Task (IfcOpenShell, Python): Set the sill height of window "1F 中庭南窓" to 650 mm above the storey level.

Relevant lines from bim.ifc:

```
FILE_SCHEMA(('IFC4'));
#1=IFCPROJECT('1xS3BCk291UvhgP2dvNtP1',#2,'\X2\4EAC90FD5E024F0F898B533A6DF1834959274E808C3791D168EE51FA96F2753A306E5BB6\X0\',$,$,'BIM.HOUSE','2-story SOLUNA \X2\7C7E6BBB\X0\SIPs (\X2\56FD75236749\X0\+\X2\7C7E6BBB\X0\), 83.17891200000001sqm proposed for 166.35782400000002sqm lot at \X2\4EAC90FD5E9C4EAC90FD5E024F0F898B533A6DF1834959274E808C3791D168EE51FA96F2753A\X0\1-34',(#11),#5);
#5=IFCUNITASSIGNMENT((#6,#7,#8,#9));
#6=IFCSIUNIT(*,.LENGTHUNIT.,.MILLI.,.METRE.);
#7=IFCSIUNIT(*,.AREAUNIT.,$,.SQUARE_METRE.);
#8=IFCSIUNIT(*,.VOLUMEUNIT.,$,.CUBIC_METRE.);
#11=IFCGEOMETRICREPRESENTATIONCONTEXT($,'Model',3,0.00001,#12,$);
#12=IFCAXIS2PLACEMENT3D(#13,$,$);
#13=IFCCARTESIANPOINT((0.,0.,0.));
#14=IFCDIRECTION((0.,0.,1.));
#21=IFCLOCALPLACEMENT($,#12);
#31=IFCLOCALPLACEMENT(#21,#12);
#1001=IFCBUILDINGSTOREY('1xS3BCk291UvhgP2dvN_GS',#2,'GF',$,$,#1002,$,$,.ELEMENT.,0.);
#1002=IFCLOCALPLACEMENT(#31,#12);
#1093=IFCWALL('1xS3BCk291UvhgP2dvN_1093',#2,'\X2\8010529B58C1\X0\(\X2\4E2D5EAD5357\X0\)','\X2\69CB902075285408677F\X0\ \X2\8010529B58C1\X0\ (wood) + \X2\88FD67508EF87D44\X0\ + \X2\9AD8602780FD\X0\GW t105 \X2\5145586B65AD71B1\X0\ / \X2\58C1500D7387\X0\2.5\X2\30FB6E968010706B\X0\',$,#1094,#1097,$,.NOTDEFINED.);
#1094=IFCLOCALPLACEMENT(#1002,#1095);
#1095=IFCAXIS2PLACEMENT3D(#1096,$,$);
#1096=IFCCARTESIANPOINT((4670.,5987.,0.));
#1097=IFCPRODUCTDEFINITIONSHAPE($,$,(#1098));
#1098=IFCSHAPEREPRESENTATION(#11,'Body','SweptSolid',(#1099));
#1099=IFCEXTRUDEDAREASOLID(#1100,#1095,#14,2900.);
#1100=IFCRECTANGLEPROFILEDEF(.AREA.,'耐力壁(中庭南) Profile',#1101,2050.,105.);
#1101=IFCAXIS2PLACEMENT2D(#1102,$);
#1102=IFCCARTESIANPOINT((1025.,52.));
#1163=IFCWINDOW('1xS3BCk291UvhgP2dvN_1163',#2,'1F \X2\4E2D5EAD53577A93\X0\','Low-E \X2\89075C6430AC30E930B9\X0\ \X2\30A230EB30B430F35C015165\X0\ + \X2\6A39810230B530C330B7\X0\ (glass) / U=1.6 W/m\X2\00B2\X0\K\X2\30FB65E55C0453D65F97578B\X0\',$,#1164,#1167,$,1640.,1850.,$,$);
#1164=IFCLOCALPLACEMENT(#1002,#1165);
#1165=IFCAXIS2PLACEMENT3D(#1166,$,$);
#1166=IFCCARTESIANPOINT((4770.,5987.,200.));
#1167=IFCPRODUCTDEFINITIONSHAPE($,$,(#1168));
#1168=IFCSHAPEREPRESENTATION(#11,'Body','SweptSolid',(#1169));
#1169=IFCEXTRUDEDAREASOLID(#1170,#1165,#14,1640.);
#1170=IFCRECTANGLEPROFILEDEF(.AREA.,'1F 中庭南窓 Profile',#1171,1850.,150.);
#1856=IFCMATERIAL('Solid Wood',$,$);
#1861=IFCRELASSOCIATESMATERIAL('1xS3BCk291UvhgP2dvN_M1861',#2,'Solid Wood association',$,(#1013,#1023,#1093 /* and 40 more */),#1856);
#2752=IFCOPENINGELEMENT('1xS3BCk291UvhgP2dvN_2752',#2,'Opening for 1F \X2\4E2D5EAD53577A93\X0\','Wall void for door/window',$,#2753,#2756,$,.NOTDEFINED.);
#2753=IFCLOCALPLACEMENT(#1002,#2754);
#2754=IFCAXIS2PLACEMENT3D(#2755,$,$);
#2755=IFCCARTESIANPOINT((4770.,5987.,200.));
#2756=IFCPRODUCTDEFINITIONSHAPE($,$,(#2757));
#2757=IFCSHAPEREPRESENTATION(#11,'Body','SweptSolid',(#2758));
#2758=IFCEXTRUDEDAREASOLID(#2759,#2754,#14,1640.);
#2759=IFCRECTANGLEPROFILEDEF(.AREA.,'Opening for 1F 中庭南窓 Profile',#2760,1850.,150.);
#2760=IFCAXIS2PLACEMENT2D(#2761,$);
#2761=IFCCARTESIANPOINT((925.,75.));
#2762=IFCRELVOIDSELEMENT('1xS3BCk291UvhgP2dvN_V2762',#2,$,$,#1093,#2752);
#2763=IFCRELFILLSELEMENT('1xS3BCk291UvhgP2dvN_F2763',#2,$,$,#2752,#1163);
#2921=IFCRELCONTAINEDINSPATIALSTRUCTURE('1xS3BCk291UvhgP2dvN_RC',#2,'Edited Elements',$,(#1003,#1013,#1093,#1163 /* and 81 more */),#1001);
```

```python
import numpy as np
import ifcopenshell
import ifcopenshell.api.geometry
import ifcopenshell.geom
import ifcopenshell.util.element
import ifcopenshell.util.placement
import ifcopenshell.util.shape
import ifcopenshell.util.unit

model = ifcopenshell.open("bim.ifc")
unit_scale = ifcopenshell.util.unit.calculate_unit_scale(model)

window = model.by_id(1163)
opening = window.FillsVoids[0].RelatingOpeningElement
storey = ifcopenshell.util.element.get_container(window, ifc_class="IfcBuildingStorey")
level = ifcopenshell.util.placement.get_local_placement(storey.ObjectPlacement)[2, 3]

# The opening's origin need not be at the sill, so measure its lowest point.
shape = ifcopenshell.geom.create_shape(ifcopenshell.geom.settings(), opening)
bottom = ifcopenshell.util.shape.get_shape_bottom_elevation(shape, shape.geometry) / unit_scale
dz = level + 0.65 / unit_scale - bottom

shift = np.array([0.0, 0.0, dz])
# The window is not placed relative to its opening, so move both.
for product in (opening, window):
    matrix = ifcopenshell.util.placement.get_local_placement(product.ObjectPlacement)
    matrix[:3, 3] += shift
    ifcopenshell.api.geometry.edit_object_placement(model, product=product, matrix=matrix, is_si=False)

print(f"moved by {dz * unit_scale:+.3f} m")

model.write("bim_edited.ifc")
```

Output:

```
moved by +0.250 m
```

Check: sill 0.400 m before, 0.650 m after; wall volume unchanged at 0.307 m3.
